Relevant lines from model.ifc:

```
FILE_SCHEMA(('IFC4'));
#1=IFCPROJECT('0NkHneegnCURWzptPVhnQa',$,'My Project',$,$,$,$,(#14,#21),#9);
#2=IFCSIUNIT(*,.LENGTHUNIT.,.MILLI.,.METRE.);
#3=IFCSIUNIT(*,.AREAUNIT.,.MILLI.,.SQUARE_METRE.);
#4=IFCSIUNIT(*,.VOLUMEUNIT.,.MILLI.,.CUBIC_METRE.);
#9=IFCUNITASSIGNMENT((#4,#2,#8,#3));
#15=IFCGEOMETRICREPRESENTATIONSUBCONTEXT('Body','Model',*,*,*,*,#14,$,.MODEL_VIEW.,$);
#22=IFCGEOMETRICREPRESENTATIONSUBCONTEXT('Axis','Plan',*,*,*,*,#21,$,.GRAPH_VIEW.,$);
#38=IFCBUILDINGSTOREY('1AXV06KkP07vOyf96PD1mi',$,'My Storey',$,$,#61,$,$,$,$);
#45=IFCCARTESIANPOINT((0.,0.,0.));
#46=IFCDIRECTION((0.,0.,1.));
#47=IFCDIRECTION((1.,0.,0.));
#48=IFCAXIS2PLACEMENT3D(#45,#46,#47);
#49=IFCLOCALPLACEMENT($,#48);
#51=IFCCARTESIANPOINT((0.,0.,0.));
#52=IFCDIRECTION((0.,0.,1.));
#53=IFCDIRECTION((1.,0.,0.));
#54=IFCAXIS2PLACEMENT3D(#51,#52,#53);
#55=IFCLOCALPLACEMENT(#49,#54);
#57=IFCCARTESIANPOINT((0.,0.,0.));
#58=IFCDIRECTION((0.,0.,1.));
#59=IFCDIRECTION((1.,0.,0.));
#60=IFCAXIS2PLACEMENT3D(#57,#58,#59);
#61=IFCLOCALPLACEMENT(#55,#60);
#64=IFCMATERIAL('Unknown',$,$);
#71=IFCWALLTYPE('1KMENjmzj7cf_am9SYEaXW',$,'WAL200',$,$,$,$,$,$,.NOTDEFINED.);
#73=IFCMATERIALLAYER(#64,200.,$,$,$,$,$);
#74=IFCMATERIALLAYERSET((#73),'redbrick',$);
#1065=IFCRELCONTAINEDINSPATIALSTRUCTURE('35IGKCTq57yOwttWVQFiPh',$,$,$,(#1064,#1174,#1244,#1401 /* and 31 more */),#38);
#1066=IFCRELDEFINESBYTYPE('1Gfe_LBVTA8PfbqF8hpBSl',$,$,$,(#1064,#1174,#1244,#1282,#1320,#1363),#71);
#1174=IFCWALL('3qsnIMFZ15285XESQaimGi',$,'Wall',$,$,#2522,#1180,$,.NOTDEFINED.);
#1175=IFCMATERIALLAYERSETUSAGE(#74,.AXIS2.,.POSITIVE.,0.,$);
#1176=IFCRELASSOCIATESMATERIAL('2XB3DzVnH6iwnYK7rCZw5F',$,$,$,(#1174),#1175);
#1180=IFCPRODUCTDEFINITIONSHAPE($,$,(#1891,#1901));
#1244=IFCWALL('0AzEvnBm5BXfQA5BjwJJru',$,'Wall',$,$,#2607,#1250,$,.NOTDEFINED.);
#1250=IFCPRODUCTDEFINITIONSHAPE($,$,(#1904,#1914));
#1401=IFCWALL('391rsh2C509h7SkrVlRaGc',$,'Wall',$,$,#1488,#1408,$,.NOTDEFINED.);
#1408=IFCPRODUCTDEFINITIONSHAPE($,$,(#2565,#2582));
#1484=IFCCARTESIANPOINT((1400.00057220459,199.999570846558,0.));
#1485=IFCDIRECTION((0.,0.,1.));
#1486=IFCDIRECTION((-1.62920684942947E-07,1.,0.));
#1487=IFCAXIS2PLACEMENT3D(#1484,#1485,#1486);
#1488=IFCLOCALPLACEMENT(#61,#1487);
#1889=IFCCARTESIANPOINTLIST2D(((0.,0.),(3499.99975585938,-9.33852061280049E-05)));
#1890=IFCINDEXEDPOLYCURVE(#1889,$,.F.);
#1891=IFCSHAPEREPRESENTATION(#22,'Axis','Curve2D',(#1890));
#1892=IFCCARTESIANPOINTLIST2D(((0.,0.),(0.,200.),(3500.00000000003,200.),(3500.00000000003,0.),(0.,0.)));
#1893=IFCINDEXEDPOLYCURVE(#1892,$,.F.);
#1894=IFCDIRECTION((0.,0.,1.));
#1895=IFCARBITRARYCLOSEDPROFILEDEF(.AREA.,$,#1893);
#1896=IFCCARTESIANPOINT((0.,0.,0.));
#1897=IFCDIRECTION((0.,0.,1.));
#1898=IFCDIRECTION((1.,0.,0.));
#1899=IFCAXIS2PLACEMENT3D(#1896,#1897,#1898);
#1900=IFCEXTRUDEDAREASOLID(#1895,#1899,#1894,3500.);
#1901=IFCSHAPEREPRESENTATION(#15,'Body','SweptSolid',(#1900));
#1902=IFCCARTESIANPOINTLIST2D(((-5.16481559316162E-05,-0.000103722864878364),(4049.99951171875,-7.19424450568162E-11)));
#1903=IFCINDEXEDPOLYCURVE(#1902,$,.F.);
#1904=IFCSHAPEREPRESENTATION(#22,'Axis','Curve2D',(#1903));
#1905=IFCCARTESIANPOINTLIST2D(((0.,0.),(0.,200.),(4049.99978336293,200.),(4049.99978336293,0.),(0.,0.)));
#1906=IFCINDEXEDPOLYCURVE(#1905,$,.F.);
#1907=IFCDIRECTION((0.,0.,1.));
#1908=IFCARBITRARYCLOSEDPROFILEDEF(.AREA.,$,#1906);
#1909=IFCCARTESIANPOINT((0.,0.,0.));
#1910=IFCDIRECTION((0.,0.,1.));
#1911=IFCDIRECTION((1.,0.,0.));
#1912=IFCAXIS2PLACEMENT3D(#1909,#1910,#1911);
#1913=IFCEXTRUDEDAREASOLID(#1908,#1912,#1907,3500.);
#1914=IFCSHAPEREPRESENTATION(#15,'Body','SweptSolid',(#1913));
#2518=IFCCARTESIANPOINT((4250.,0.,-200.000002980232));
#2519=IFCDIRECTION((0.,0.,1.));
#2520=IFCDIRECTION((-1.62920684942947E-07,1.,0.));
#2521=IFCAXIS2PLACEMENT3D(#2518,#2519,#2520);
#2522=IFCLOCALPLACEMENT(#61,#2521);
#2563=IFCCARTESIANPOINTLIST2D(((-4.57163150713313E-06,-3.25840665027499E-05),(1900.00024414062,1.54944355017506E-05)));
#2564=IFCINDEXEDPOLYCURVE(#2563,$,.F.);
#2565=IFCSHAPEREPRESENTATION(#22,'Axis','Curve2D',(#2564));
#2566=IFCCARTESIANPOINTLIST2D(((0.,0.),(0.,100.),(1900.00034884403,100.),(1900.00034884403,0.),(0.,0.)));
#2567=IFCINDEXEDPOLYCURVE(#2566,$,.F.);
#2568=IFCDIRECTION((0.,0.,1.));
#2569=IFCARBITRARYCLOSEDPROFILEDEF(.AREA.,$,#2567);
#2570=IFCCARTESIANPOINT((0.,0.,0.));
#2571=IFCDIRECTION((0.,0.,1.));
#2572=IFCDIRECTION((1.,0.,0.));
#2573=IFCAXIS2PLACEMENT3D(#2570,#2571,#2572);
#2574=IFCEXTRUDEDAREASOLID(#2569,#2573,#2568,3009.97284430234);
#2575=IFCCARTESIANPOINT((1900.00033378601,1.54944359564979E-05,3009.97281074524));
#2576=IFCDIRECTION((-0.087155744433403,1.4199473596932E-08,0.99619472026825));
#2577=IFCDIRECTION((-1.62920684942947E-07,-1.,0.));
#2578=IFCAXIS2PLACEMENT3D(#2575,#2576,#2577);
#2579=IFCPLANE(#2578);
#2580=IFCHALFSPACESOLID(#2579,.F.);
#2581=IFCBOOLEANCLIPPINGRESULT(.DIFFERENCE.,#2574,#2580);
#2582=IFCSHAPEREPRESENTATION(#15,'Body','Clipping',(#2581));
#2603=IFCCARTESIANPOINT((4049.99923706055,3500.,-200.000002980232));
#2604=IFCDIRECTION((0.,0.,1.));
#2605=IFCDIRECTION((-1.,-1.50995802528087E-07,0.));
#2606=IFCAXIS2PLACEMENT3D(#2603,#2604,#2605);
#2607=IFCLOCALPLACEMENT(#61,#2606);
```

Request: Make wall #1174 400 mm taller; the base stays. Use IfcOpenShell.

```python
import ifcopenshell
import ifcopenshell.geom
import ifcopenshell.util.representation
import ifcopenshell.util.shape

model = ifcopenshell.open("model.ifc")
settings = ifcopenshell.geom.settings()


def volume(element):
    """Net volume in cubic metres, openings subtracted."""
    shape = ifcopenshell.geom.create_shape(settings, element)
    return ifcopenshell.util.shape.get_volume(shape.geometry)


wall = model.by_guid("3qsnIMFZ15285XESQaimGi")
before = volume(wall)

body = ifcopenshell.util.representation.get_representation(wall, "Model", "Body")
solid = body.Items[0]
old_height = solid.Depth
solid.Depth += 400.0
after = volume(wall)

print(f"height {old_height:g} -> {solid.Depth:g}, volume {before:.3f} -> {after:.3f} m3")

model.write("model_rev.ifc")
```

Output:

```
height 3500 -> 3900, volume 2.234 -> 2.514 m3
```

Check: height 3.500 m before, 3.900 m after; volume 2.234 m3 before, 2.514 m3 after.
